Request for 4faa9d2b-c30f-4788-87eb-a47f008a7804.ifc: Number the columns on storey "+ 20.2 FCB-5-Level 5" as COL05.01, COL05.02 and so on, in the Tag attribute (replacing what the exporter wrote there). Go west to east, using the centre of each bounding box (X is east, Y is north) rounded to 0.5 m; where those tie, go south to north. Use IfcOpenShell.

First a look at what the model holds.

```python
import ifcopenshell
import ifcopenshell.util.element
import ifcopenshell.util.placement

model = ifcopenshell.open("4faa9d2b-c30f-4788-87eb-a47f008a7804.ifc")
print(model.schema)
storey = next(s for s in model.by_type("IfcBuildingStorey") if s.Name == "+ 20.2 FCB-5-Level 5")
columns = [e for e in ifcopenshell.util.element.get_decomposition(storey) if e.is_a("IfcColumn")]
for e in sorted(columns, key=lambda e: e.id()):
    origin = ifcopenshell.util.placement.get_local_placement(e.ObjectPlacement)[:3, 3]
    print(e.id(), e.Tag, e.Name, origin.round(2) + 0.0, sep=" | ")
```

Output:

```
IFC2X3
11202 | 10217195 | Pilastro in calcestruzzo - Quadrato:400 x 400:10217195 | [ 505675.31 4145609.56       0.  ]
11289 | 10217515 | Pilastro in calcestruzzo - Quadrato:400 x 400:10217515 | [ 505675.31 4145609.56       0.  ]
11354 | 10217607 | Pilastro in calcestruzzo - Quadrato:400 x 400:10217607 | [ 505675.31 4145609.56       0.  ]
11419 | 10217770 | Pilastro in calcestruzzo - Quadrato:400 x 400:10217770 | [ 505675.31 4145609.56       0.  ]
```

```python
import ifcopenshell
import ifcopenshell.geom
import ifcopenshell.util.element
import ifcopenshell.util.shape

model = ifcopenshell.open("4faa9d2b-c30f-4788-87eb-a47f008a7804.ifc")
settings = ifcopenshell.geom.settings()
settings.set("use-world-coords", True)


def centre(element):
    shape = ifcopenshell.geom.create_shape(settings, element)
    return ifcopenshell.util.shape.get_bbox_centroid(shape.geometry)


storey = next(s for s in model.by_type("IfcBuildingStorey") if s.Name == "+ 20.2 FCB-5-Level 5")
columns = [e for e in ifcopenshell.util.element.get_decomposition(storey) if e.is_a("IfcColumn")]

# Insertion points can sit at a corner or the storey origin, so sort by the geometry (in metres).
centres = {e: centre(e) for e in columns}
columns.sort(key=lambda e: (round(centres[e][0] / 0.5), centres[e][1]))

for i, e in enumerate(columns, start=1):
    number = f"COL05.{i:02d}"
    e.Tag = number
    print(e.id(), number)

model.write("4faa9d2b-c30f-4788-87eb-a47f008a7804_updated.ifc")
```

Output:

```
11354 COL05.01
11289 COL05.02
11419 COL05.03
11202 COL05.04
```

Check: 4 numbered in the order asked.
